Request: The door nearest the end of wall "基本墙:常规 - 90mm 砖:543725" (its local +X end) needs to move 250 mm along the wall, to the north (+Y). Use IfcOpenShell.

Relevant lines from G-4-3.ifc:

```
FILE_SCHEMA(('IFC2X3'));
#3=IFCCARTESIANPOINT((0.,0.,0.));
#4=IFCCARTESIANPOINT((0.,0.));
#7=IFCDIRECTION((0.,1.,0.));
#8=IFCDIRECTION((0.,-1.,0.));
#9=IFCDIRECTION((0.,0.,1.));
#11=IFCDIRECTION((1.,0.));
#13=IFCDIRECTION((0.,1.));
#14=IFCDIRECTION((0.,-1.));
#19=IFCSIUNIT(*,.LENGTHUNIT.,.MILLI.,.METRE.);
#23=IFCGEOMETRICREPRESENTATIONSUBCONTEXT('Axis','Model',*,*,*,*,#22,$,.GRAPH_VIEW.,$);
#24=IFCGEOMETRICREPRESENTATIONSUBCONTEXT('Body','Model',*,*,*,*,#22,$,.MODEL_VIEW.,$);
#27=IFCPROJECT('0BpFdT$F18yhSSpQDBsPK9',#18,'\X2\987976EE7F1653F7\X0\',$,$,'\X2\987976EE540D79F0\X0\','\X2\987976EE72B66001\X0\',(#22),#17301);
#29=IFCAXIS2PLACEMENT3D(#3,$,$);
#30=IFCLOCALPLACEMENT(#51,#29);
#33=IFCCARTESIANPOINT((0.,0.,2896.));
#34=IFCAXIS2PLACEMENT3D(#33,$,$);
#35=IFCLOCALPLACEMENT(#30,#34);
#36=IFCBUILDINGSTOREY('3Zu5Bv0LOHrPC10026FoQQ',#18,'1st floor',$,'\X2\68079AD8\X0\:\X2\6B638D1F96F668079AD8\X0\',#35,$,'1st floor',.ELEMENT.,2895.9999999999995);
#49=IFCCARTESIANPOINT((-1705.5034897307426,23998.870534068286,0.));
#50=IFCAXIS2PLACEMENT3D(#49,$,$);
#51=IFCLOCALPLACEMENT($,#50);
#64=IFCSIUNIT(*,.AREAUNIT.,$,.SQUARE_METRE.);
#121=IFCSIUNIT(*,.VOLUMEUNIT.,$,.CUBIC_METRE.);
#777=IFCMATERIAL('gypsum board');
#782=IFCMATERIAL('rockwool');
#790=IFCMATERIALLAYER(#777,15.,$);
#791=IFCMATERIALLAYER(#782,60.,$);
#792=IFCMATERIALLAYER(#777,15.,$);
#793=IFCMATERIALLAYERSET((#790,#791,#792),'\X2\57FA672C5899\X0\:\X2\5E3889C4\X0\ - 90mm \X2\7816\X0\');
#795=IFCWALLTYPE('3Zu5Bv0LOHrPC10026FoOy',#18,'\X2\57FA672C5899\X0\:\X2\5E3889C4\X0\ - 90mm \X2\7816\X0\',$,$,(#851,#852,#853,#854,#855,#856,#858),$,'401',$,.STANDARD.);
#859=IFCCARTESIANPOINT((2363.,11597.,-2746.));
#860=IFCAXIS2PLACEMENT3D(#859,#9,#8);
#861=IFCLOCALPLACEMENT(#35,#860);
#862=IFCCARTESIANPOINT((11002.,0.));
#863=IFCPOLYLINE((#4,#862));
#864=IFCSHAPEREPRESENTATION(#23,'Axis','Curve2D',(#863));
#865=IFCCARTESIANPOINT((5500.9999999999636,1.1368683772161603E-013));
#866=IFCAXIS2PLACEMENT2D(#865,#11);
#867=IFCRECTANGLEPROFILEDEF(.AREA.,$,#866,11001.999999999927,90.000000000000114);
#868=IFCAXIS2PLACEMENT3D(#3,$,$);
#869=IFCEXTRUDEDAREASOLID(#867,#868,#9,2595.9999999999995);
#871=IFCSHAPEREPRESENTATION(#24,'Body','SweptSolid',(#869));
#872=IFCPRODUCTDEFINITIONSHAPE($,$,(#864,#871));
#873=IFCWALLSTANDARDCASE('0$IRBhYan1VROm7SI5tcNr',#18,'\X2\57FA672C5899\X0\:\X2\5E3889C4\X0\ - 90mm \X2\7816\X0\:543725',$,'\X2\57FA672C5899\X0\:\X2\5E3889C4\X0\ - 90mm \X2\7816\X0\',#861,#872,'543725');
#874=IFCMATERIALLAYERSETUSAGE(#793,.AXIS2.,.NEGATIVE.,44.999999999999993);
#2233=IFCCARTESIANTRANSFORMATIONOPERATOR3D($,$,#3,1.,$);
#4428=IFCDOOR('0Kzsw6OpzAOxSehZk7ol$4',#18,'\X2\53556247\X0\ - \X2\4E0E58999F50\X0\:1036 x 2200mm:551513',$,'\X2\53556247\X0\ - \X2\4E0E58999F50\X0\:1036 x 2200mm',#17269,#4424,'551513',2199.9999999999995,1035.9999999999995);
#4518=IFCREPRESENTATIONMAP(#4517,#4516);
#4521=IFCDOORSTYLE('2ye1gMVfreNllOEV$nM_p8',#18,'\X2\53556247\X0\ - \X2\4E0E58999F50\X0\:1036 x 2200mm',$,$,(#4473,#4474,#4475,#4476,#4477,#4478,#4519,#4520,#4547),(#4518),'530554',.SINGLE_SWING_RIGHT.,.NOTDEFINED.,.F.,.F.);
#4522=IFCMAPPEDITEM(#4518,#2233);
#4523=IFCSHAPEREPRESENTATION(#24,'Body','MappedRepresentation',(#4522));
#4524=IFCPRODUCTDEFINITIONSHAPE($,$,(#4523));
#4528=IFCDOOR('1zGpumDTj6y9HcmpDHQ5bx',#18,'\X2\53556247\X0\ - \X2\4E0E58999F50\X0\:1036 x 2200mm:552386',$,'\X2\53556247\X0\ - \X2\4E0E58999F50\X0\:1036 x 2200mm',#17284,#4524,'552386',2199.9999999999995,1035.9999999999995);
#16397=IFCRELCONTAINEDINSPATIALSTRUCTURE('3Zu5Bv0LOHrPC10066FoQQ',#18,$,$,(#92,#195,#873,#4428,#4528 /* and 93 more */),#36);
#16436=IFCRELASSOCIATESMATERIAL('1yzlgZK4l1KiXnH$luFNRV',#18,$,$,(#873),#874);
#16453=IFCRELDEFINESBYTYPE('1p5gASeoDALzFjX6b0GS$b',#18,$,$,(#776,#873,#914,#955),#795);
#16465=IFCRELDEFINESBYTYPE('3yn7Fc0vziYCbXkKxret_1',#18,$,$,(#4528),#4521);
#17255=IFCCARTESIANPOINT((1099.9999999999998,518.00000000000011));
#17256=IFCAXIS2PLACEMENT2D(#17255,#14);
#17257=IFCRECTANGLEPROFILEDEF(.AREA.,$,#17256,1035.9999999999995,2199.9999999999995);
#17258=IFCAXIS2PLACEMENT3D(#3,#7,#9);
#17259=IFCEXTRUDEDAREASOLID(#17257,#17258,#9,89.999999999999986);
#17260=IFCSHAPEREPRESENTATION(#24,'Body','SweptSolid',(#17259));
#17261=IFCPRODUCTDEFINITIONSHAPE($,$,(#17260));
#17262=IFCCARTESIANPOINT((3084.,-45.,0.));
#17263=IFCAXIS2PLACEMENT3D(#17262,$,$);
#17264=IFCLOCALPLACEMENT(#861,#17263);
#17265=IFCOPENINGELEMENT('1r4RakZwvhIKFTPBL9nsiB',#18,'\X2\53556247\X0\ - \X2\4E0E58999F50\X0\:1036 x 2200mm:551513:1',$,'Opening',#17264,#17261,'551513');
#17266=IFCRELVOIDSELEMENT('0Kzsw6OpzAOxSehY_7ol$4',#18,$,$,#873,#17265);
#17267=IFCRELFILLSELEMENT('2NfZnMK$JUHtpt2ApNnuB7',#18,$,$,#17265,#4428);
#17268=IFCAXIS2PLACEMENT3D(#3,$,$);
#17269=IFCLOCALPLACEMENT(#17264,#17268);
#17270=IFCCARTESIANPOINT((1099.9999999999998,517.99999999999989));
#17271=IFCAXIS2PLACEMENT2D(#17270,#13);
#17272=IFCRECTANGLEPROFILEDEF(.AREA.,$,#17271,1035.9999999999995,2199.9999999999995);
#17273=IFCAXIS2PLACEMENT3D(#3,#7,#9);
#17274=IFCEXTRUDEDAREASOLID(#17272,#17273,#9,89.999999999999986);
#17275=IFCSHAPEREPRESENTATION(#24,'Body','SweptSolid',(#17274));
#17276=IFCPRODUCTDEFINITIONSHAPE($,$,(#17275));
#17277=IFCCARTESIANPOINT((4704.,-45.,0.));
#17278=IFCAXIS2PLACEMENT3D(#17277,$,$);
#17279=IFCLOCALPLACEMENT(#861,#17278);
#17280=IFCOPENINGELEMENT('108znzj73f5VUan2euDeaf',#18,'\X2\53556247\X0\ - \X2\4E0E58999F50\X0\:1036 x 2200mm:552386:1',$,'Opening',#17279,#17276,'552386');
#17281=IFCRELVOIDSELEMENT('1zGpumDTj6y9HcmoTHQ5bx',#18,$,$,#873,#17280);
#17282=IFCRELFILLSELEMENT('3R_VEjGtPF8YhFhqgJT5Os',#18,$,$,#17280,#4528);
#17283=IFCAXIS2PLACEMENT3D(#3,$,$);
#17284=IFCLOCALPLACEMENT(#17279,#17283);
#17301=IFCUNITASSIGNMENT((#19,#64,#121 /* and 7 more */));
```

```python
import ifcopenshell
import ifcopenshell.api.geometry
import ifcopenshell.util.placement
import ifcopenshell.util.unit

model = ifcopenshell.open("G-4-3.ifc")
unit_scale = ifcopenshell.util.unit.calculate_unit_scale(model)

door = model.by_guid("1zGpumDTj6y9HcmpDHQ5bx")
opening = door.FillsVoids[0].RelatingOpeningElement
wall = opening.VoidsElements[0].RelatingBuildingElement

wall_matrix = ifcopenshell.util.placement.get_local_placement(wall.ObjectPlacement)
shift = wall_matrix[:3, 0] * -0.25 / unit_scale
before = ifcopenshell.util.placement.get_local_placement(door.ObjectPlacement)[:3, 3].copy()

# The door is placed relative to its opening, so it follows when the opening moves.
matrix = ifcopenshell.util.placement.get_local_placement(opening.ObjectPlacement)
matrix[:3, 3] += shift
ifcopenshell.api.geometry.edit_object_placement(
    model, product=opening, matrix=matrix, is_si=False, should_transform_children=True
)

after = ifcopenshell.util.placement.get_local_placement(door.ObjectPlacement)[:3, 3]
print("door moved by", (after - before).round(3) + 0.0)

model.write("G-4-3-out.ifc")
```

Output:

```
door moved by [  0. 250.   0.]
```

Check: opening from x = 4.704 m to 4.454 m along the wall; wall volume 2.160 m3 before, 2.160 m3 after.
